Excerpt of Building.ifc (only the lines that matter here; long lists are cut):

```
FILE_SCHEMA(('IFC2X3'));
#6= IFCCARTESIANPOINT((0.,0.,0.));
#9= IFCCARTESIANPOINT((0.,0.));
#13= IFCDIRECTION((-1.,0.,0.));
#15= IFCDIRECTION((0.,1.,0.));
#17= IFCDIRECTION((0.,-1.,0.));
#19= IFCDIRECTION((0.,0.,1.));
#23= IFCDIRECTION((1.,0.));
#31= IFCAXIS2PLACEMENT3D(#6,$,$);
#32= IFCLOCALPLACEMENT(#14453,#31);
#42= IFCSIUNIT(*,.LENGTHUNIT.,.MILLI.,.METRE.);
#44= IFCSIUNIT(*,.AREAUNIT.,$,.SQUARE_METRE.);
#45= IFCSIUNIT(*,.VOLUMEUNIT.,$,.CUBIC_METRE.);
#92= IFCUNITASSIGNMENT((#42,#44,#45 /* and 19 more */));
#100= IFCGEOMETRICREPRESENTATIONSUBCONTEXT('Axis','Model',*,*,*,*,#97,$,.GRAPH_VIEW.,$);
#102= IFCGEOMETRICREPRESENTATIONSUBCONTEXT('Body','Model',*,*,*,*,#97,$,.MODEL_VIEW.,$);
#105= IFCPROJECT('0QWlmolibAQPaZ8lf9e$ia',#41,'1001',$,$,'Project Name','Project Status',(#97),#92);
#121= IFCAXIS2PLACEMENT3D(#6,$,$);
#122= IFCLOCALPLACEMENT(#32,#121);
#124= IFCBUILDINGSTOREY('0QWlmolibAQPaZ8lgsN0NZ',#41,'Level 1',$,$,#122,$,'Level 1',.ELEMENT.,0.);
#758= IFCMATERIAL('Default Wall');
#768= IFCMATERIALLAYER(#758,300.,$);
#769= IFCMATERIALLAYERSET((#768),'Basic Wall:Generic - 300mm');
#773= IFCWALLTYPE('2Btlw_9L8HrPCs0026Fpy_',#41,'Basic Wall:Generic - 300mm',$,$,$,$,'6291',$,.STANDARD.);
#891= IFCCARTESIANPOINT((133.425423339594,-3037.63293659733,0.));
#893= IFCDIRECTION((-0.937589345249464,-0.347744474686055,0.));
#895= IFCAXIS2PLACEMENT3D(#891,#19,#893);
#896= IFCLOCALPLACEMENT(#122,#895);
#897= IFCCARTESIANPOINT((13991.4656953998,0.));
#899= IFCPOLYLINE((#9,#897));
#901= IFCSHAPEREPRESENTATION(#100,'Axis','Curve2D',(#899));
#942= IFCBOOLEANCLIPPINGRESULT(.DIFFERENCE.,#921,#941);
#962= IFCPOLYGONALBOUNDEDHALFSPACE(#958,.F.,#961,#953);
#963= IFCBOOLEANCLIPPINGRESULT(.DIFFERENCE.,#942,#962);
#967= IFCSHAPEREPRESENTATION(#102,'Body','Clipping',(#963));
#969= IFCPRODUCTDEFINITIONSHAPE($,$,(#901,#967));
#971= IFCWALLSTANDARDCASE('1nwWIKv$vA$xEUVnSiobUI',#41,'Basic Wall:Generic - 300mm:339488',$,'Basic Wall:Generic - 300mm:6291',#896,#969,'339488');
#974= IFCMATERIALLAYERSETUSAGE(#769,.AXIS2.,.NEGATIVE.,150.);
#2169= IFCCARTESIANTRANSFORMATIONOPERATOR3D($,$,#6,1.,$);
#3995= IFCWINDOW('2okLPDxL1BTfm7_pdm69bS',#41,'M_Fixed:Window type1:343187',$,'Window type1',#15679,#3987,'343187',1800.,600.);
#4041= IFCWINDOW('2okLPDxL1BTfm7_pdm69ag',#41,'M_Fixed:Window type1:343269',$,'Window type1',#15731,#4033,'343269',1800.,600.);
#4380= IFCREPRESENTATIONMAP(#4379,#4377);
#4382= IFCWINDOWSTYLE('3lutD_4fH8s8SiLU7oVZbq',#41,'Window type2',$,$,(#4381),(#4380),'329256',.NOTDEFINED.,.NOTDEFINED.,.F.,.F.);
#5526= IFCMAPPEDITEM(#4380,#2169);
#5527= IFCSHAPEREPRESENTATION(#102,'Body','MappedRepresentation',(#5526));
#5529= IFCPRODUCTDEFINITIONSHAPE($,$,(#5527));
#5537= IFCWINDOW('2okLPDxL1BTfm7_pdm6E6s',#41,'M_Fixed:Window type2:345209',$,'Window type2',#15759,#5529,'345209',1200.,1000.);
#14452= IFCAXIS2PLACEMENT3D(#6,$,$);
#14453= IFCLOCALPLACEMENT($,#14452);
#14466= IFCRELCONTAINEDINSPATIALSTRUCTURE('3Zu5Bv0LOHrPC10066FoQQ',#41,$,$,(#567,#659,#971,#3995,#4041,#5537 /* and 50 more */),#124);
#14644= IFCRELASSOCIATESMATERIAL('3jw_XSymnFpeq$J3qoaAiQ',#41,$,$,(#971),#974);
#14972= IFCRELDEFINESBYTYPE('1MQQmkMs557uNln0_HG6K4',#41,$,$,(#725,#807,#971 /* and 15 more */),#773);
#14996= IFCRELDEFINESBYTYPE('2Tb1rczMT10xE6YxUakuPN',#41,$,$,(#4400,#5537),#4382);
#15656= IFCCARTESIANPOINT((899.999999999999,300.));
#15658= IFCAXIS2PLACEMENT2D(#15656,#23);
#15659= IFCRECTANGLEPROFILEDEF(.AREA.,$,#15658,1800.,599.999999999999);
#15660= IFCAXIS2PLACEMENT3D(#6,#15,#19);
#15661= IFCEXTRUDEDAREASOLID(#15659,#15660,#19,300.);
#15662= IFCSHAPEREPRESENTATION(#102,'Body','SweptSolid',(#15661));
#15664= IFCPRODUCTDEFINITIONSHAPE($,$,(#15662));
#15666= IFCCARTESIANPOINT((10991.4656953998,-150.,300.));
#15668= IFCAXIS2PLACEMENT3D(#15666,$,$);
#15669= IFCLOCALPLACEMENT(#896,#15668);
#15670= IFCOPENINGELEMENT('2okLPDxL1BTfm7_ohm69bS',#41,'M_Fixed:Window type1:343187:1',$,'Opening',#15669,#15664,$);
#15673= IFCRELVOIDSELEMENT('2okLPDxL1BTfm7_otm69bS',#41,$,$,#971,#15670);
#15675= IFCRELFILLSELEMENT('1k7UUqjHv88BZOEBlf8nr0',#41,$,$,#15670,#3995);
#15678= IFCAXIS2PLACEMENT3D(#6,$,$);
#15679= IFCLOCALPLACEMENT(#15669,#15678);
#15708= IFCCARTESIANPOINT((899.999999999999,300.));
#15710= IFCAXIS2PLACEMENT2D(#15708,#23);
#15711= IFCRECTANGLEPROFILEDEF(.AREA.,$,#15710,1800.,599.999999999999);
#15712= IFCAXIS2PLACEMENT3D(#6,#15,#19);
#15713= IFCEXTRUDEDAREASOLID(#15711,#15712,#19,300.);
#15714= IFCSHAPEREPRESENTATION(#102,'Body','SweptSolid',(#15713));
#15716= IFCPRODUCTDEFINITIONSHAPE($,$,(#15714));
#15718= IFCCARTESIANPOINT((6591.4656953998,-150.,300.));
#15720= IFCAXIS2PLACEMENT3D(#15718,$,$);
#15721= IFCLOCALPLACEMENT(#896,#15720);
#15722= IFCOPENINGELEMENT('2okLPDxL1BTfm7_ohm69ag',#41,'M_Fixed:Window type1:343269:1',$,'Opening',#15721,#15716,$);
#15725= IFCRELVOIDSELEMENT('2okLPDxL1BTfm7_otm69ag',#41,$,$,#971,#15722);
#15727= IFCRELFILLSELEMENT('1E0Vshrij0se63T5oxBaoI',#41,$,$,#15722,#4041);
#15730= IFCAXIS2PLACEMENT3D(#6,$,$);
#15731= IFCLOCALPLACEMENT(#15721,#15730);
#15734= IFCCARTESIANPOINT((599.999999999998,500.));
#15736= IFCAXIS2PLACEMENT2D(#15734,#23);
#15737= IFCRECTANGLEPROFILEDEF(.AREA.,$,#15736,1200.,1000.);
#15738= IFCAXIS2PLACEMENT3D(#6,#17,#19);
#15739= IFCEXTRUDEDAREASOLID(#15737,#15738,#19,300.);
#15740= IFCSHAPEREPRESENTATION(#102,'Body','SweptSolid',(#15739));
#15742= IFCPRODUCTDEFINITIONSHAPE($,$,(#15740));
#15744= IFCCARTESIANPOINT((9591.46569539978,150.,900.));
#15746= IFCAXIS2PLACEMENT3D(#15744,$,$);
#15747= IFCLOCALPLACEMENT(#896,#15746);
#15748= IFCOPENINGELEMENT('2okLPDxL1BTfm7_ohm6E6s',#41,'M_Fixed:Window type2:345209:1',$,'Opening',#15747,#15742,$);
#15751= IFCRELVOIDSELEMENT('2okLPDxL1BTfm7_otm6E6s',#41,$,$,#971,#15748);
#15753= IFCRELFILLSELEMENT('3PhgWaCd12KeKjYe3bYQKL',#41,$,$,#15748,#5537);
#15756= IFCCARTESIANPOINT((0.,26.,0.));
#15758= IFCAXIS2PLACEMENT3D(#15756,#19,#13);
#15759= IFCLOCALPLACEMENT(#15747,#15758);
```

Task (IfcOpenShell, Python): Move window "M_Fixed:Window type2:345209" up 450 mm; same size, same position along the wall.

```python
import numpy as np
import ifcopenshell
import ifcopenshell.api.geometry
import ifcopenshell.util.placement
import ifcopenshell.util.unit

model = ifcopenshell.open("Building.ifc")
unit_scale = ifcopenshell.util.unit.calculate_unit_scale(model)

window = model.by_guid("2okLPDxL1BTfm7_pdm6E6s")
opening = window.FillsVoids[0].RelatingOpeningElement
dz = 0.45 / unit_scale

shift = np.array([0.0, 0.0, dz])
# The window is placed relative to its opening, so it follows when the opening moves.
matrix = ifcopenshell.util.placement.get_local_placement(opening.ObjectPlacement)
matrix[:3, 3] += shift
ifcopenshell.api.geometry.edit_object_placement(
    model, product=opening, matrix=matrix, is_si=False, should_transform_children=True
)

print(f"moved by {dz * unit_scale:+.3f} m")

model.write("Building_v2.ifc")
```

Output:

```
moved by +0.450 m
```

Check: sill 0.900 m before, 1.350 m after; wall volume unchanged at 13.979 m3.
